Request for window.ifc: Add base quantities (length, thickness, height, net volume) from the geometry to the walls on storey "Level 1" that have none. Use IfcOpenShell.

First a look at what the model holds.

```python
import ifcopenshell
import ifcopenshell.util.element
import ifcopenshell.util.unit

model = ifcopenshell.open("window.ifc")
print(model.schema)
for unit_type in ("LENGTHUNIT", "AREAUNIT", "VOLUMEUNIT"):
    print(unit_type, ifcopenshell.util.unit.calculate_unit_scale(model, unit_type))
storey = next(s for s in model.by_type("IfcBuildingStorey") if s.Name == "Level 1")
walls = [e for e in ifcopenshell.util.element.get_decomposition(storey) if e.is_a("IfcWall")]
for e in sorted(walls, key=lambda e: e.id()):
    print(e.id(), e.is_a(), e.Name, list(ifcopenshell.util.element.get_psets(e, qtos_only=True)), sep=" | ")
```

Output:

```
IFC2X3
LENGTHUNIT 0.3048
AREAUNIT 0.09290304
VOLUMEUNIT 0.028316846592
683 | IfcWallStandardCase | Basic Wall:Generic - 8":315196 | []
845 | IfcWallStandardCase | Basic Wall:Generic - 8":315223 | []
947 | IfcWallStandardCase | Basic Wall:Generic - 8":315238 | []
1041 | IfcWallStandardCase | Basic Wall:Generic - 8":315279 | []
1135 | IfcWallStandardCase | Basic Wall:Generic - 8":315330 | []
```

```python
import ifcopenshell
import ifcopenshell.api.pset
import ifcopenshell.geom
import ifcopenshell.util.element
import ifcopenshell.util.shape
import ifcopenshell.util.unit

model = ifcopenshell.open("window.ifc")
unit_scale = ifcopenshell.util.unit.calculate_unit_scale(model)
volume_scale = ifcopenshell.util.unit.calculate_unit_scale(model, "VOLUMEUNIT")
settings = ifcopenshell.geom.settings()

storey = next(s for s in model.by_type("IfcBuildingStorey") if s.Name == "Level 1")
walls = [e for e in ifcopenshell.util.element.get_decomposition(storey) if e.is_a("IfcWall")]

for e in sorted(walls, key=lambda e: e.id()):
    if ifcopenshell.util.element.get_psets(e, qtos_only=True, should_inherit=False):
        continue
    # Geometry comes back in metres, in the element's own axes.
    shape = ifcopenshell.geom.create_shape(settings, e)
    values = {
        "Length": ifcopenshell.util.shape.get_x(shape.geometry) / unit_scale,
        "Width": ifcopenshell.util.shape.get_y(shape.geometry) / unit_scale,
        "Height": ifcopenshell.util.shape.get_z(shape.geometry) / unit_scale,
        "NetVolume": ifcopenshell.util.shape.get_volume(shape.geometry) / volume_scale,
    }
    qto = ifcopenshell.api.pset.add_qto(model, product=e, name="BaseQuantities")
    ifcopenshell.api.pset.edit_qto(model, qto=qto, properties=values)
    print(e.id(), {k: round(v, 3) for k, v in values.items()})

model.write("window_edited.ifc")
```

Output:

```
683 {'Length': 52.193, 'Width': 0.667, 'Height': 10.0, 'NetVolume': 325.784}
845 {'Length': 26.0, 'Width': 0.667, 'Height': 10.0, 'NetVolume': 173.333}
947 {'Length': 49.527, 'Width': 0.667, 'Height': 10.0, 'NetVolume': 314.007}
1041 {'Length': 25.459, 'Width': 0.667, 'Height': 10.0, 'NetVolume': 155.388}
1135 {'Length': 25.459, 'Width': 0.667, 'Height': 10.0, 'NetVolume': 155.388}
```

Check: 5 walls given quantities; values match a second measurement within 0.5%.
